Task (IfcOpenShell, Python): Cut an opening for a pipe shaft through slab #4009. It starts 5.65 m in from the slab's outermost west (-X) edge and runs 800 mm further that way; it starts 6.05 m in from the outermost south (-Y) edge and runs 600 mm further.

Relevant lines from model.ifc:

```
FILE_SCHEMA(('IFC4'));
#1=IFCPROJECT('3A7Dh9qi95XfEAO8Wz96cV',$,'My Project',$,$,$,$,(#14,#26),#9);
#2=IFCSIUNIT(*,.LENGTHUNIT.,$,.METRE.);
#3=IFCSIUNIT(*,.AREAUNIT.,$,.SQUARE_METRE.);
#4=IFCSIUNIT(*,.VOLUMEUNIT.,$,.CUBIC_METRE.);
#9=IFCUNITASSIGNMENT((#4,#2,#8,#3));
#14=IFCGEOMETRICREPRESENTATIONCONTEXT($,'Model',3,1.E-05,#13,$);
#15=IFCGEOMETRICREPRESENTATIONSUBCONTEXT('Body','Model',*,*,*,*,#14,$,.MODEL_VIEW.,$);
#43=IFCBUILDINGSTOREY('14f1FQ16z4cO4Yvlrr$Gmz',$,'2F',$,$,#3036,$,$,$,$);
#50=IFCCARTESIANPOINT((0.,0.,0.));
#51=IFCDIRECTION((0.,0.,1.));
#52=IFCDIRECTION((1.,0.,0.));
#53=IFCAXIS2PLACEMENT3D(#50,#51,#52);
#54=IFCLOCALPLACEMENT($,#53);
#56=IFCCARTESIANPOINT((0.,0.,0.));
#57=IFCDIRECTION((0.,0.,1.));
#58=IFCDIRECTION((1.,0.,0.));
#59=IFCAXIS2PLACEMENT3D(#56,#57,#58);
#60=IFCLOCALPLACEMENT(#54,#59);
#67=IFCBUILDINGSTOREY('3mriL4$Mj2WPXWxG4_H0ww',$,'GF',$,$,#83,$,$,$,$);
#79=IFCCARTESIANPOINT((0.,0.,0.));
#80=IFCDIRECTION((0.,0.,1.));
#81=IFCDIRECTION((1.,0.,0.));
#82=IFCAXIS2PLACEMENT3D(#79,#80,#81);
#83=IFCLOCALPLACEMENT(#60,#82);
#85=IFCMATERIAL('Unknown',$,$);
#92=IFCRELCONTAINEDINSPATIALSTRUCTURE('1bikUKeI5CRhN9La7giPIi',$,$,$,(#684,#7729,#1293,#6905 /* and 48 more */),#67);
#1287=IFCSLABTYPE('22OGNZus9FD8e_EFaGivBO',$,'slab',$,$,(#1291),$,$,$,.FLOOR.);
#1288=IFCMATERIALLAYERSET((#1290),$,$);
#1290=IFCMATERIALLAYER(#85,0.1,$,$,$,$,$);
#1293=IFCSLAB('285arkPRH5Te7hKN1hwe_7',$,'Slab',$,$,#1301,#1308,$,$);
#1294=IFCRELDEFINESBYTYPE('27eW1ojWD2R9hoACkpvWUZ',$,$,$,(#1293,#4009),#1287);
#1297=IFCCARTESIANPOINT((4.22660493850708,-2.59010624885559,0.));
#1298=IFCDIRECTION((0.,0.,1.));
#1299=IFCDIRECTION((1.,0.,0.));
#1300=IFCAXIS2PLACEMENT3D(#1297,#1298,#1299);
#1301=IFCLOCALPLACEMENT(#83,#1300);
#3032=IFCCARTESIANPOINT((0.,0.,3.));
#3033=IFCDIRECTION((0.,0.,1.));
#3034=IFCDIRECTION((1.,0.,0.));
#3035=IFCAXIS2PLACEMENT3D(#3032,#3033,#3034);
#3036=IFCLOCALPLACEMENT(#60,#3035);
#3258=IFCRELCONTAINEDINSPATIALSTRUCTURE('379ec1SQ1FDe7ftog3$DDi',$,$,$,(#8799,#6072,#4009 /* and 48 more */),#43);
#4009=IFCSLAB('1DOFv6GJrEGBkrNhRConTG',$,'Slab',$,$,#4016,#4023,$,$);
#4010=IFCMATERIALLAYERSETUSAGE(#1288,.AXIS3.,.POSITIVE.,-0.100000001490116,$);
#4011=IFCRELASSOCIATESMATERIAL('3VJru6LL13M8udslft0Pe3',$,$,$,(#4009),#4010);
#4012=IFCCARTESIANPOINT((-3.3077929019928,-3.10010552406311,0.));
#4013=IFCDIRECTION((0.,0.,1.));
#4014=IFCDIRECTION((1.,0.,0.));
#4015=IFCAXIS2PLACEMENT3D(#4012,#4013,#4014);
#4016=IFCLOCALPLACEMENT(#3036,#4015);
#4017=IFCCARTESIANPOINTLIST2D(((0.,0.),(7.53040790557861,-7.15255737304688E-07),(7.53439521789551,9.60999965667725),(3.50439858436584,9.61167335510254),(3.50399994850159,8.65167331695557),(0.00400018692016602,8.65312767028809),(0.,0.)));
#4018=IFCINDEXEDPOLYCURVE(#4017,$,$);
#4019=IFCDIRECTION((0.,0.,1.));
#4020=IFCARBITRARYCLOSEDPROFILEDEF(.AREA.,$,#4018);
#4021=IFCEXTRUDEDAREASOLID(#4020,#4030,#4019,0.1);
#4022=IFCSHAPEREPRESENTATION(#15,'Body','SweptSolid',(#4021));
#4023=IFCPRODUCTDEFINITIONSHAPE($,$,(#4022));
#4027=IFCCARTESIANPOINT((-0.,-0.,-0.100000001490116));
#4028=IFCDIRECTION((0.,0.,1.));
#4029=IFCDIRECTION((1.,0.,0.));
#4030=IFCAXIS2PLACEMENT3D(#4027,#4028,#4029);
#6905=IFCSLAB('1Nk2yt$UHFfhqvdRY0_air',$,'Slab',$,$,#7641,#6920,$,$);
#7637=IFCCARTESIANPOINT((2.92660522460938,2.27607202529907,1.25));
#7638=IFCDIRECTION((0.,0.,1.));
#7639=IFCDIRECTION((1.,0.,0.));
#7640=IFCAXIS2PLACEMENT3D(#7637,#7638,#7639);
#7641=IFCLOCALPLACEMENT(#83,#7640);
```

```python
import numpy as np
import ifcopenshell
import ifcopenshell.api.feature
import ifcopenshell.api.geometry
import ifcopenshell.api.root
import ifcopenshell.geom
import ifcopenshell.util.placement
import ifcopenshell.util.representation
import ifcopenshell.util.shape
import ifcopenshell.util.unit

model = ifcopenshell.open("model.ifc")
unit_scale = ifcopenshell.util.unit.calculate_unit_scale(model)
settings = ifcopenshell.geom.settings()


def volume(element):
    """Net volume in cubic metres, openings subtracted."""
    shape = ifcopenshell.geom.create_shape(settings, element)
    return ifcopenshell.util.shape.get_volume(shape.geometry)


slab = model.by_guid("1DOFv6GJrEGBkrNhRConTG")
before = volume(slab)

# Extent in the slab's own axes, in metres. The edges named are its -X and -Y sides.
slab_shape = ifcopenshell.geom.create_shape(settings, slab)
vertices = ifcopenshell.util.shape.get_vertices(slab_shape.geometry)
x_min, y_min, bottom = vertices.min(axis=0)
top = vertices[:, 2].max()

opening = ifcopenshell.api.root.create_entity(model, ifc_class="IfcOpeningElement", name="Pipe shaft opening", predefined_type="OPENING")
context = ifcopenshell.util.representation.get_context(model, "Model", "Body", "MODEL_VIEW")
width, depth = 0.8, 0.6
outline = [(0.0, 0.0), (width, 0.0), (width, depth), (0.0, depth), (0.0, 0.0)]
# Overshoot both faces by 50 mm so the cut is clean.
shape = ifcopenshell.api.geometry.add_slab_representation(
    model, context=context, depth=top - bottom + 0.1, polyline=outline
)
ifcopenshell.api.geometry.assign_representation(model, product=opening, representation=shape)

matrix = ifcopenshell.util.placement.get_local_placement(slab.ObjectPlacement)
matrix[:, 3] = matrix @ np.append(np.array([x_min + 5.65, y_min + 6.05, bottom - 0.05]) / unit_scale, 1.0)
ifcopenshell.api.geometry.edit_object_placement(model, product=opening, matrix=matrix, is_si=False)
ifcopenshell.api.feature.add_feature(model, feature=opening, element=slab)

after = volume(slab)

print(f"slab volume {before:.3f} -> {after:.3f} m3")

model.write("model_v2.ifc")
```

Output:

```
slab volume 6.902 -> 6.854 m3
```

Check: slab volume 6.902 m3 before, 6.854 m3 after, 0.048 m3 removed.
